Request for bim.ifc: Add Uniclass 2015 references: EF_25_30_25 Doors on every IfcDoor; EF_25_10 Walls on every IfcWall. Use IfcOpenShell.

First a look at what the model holds.

```python
import ifcopenshell

model = ifcopenshell.open("bim.ifc")
print(model.schema)
print("classifications:", [c.Name for c in model.by_type("IfcClassification")])
for ifc_class in ("IfcDoor", "IfcRoof", "IfcStair", "IfcWall", "IfcWindow"):
    print(ifc_class, len(model.by_type(ifc_class)))
```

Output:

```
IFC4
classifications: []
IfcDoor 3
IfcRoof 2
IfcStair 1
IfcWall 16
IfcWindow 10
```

```python
import ifcopenshell
import ifcopenshell.api.classification

model = ifcopenshell.open("bim.ifc")

system = ifcopenshell.api.classification.add_classification(model, classification="Uniclass 2015")

codes = {
    "IfcDoor": ("EF_25_30_25", "Doors"),
    "IfcWall": ("EF_25_10", "Walls"),
}
for ifc_class, (code, name) in codes.items():
    products = model.by_type(ifc_class)
    ifcopenshell.api.classification.add_reference(
        model, products=products, classification=system, identification=code, name=name
    )
    print(code, len(products))

model.write("bim_rev.ifc")
```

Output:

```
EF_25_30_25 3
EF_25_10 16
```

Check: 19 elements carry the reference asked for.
